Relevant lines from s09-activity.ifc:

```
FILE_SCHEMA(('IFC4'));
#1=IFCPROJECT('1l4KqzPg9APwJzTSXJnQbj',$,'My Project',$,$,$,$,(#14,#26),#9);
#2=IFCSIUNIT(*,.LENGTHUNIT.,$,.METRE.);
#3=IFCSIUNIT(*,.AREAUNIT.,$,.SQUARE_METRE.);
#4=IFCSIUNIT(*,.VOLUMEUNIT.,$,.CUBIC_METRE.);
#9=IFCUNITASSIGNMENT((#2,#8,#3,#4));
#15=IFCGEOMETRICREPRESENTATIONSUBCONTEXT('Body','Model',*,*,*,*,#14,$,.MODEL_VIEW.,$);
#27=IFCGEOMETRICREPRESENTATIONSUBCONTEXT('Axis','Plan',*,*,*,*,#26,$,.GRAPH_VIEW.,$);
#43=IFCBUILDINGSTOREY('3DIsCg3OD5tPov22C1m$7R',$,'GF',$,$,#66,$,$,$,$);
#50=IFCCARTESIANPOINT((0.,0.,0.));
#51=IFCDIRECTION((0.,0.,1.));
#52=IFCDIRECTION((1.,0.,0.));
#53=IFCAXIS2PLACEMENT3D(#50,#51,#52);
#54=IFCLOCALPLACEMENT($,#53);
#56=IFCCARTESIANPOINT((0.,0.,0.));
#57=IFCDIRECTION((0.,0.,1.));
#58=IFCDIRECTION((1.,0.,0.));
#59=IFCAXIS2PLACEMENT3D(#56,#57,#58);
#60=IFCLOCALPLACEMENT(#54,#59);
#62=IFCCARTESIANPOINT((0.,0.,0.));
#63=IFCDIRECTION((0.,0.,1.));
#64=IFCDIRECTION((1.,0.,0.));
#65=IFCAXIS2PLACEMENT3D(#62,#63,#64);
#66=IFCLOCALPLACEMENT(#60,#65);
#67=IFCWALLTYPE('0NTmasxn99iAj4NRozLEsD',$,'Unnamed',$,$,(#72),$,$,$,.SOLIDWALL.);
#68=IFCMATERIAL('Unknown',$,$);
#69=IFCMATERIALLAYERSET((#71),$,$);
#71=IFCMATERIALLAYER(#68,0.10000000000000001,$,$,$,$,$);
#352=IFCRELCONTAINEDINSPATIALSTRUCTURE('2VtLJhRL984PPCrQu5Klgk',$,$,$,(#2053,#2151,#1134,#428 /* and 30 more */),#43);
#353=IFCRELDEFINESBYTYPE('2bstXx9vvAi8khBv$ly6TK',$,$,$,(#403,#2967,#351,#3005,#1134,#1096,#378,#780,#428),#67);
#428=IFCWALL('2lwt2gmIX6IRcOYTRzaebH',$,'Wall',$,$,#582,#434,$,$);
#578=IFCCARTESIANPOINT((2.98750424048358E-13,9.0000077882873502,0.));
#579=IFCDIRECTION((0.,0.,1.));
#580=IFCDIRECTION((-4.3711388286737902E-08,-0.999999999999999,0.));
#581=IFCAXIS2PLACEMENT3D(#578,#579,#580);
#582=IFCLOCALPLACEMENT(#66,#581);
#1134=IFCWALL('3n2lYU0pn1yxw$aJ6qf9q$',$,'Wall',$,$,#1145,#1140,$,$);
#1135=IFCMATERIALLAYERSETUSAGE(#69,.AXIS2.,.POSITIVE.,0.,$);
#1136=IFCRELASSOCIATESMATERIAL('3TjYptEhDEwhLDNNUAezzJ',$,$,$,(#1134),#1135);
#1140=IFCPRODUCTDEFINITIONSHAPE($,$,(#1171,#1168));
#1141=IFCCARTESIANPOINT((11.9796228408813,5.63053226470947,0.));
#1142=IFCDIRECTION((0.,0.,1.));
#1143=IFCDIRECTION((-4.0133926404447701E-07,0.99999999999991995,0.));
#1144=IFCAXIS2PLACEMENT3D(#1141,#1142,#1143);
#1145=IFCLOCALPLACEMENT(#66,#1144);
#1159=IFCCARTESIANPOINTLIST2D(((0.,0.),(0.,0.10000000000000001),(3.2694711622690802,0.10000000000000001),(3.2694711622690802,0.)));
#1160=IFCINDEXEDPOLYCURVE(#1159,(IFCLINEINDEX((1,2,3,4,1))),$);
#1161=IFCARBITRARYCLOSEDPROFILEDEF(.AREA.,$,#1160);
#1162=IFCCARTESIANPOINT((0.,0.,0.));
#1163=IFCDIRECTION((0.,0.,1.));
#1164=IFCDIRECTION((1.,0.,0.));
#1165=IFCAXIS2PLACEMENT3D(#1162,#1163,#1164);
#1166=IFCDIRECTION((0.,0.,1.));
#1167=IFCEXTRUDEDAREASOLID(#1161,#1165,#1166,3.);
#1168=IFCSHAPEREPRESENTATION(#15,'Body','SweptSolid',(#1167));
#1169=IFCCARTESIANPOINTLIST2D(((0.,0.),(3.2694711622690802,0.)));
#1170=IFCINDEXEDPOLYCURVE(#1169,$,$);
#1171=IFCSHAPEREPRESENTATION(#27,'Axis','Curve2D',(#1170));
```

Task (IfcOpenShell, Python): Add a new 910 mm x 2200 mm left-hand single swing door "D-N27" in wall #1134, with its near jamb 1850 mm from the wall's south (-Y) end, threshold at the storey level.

```python
import numpy as np
import ifcopenshell
import ifcopenshell.api.feature
import ifcopenshell.api.geometry
import ifcopenshell.api.root
import ifcopenshell.api.spatial
import ifcopenshell.geom
import ifcopenshell.util.element
import ifcopenshell.util.placement
import ifcopenshell.util.representation
import ifcopenshell.util.shape
import ifcopenshell.util.unit

model = ifcopenshell.open("s09-activity.ifc")
unit_scale = ifcopenshell.util.unit.calculate_unit_scale(model)
settings = ifcopenshell.geom.settings()


def volume(element):
    """Net volume in cubic metres, openings subtracted."""
    shape = ifcopenshell.geom.create_shape(settings, element)
    return ifcopenshell.util.shape.get_volume(shape.geometry)


wall = model.by_id(1134)
storey = ifcopenshell.util.element.get_container(wall, ifc_class="IfcBuildingStorey")
context = ifcopenshell.util.representation.get_context(model, "Model", "Body", "MODEL_VIEW")
before = volume(wall)

width, height, from_end, sill = 0.91, 2.2, 1.85, 0.0  # metres

# The wall runs along its own X axis, and the end named is its -X end.
wall_shape = ifcopenshell.geom.create_shape(settings, wall)
x, y, z = ifcopenshell.util.shape.get_vertices(wall_shape.geometry).T
start = x.min() + from_end
face, thickness = float(y.min()), float(y.max() - y.min())
wall_matrix = ifcopenshell.util.placement.get_local_placement(wall.ObjectPlacement)
level = ifcopenshell.util.placement.get_local_placement(storey.ObjectPlacement)[2, 3]


def in_wall(x, y):
    """Placement at x, y metres in the wall's axes, at sill height."""
    matrix = wall_matrix.copy()
    matrix[:, 3] = wall_matrix @ np.array([x / unit_scale, y / unit_scale, 0.0, 1.0])
    matrix[2, 3] = level + sill / unit_scale
    return matrix


# Opening: a box that overshoots both wall faces by 50 mm.
opening = ifcopenshell.api.root.create_entity(model, ifc_class="IfcOpeningElement", predefined_type="OPENING")
box = ifcopenshell.api.geometry.add_wall_representation(
    model, context=context, length=width, height=height, thickness=thickness + 0.1
)
ifcopenshell.api.geometry.assign_representation(model, product=opening, representation=box)
ifcopenshell.api.geometry.edit_object_placement(model, product=opening, matrix=in_wall(start, face - 0.05), is_si=False)
ifcopenshell.api.feature.add_feature(model, feature=opening, element=wall)

door = ifcopenshell.api.root.create_entity(model, ifc_class="IfcDoor", name="D-N27", predefined_type="DOOR")
door.OverallWidth, door.OverallHeight = width / unit_scale, height / unit_scale
door.OperationType = "SINGLE_SWING_LEFT"
body = ifcopenshell.api.geometry.add_door_representation(
    model,
    context=context,
    overall_width=door.OverallWidth,
    overall_height=door.OverallHeight,
    operation_type="SINGLE_SWING_LEFT",
    lining_properties={"LiningDepth": thickness / unit_scale, "ThresholdDepth": thickness / unit_scale},
)
ifcopenshell.api.geometry.assign_representation(model, product=door, representation=body)
ifcopenshell.api.spatial.assign_container(model, products=[door], relating_structure=storey)
ifcopenshell.api.feature.add_filling(model, opening=opening, element=door)

# The lining spans the wall, so the door starts at the wall face.
ifcopenshell.api.geometry.edit_object_placement(model, product=door, matrix=in_wall(start, face), is_si=False)

after = volume(wall)

print(f"wall volume {before:.3f} -> {after:.3f} m3")

model.write("s09-activity_updated.ifc")
```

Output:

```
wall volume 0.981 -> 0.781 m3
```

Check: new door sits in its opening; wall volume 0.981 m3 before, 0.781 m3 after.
